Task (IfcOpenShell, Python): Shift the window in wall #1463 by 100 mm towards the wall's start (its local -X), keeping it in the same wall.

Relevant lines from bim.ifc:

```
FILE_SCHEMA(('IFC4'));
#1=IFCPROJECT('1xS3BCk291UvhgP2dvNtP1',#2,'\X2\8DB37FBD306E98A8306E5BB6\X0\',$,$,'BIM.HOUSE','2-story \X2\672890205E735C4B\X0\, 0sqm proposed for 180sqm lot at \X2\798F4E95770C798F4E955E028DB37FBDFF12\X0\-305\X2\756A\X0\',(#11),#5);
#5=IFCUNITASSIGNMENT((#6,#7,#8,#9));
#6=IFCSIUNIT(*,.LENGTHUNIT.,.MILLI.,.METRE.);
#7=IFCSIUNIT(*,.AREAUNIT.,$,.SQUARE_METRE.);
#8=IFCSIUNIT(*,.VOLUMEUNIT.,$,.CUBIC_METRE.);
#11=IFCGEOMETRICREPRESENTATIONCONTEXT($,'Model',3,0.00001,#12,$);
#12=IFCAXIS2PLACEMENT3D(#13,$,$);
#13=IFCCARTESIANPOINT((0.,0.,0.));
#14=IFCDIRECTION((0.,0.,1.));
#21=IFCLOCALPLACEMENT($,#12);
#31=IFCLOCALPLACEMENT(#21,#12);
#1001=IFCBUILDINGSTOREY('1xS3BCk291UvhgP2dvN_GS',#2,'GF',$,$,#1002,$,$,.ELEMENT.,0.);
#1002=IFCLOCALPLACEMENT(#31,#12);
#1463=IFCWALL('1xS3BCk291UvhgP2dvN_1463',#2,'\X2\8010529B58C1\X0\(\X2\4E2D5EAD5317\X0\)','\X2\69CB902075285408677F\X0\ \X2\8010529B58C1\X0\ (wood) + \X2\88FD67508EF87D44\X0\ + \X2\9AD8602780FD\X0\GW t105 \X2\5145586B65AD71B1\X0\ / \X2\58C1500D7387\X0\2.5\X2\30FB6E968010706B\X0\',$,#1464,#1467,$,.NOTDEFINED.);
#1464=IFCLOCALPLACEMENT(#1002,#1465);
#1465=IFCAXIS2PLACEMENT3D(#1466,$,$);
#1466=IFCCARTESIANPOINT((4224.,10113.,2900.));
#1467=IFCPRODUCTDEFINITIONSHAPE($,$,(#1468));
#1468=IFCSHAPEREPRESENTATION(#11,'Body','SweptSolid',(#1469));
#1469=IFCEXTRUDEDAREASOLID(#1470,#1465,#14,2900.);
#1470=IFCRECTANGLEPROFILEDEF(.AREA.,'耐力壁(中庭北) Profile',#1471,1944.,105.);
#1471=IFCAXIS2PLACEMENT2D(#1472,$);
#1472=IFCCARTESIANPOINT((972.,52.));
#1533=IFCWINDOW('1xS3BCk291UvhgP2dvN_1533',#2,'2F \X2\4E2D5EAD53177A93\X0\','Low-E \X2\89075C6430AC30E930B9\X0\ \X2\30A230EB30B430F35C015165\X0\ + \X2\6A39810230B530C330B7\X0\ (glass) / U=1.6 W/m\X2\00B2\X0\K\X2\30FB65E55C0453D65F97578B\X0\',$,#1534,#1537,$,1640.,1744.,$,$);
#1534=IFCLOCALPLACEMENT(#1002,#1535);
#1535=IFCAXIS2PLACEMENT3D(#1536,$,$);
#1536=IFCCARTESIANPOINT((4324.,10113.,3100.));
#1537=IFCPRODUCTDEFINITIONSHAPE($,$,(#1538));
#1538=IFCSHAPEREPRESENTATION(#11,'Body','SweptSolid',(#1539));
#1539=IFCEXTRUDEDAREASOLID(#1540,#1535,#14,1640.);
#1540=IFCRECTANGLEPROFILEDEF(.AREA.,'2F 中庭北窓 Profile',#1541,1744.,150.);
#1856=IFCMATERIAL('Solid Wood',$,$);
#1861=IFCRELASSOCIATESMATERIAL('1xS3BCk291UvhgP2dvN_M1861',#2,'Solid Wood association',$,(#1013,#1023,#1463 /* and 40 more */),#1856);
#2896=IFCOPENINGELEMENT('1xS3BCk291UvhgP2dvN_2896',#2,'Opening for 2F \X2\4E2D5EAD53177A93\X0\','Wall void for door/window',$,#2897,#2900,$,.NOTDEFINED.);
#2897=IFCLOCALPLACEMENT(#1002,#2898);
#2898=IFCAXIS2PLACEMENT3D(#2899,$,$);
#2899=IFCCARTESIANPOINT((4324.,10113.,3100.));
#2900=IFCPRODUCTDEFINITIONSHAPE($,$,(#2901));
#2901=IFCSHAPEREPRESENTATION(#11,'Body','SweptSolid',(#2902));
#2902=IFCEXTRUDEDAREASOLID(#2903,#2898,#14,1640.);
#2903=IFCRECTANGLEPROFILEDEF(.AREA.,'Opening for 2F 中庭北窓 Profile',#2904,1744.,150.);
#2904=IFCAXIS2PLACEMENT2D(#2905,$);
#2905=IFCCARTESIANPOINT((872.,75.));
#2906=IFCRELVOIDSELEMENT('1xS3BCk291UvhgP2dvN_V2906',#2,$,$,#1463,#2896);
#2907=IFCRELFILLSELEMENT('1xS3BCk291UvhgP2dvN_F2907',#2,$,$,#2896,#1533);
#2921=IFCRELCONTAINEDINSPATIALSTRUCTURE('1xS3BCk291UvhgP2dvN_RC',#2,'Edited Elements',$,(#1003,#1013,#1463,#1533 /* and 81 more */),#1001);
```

```python
import ifcopenshell
import ifcopenshell.api.geometry
import ifcopenshell.util.placement
import ifcopenshell.util.unit

model = ifcopenshell.open("bim.ifc")
unit_scale = ifcopenshell.util.unit.calculate_unit_scale(model)

window = model.by_id(1533)
opening = window.FillsVoids[0].RelatingOpeningElement
wall = opening.VoidsElements[0].RelatingBuildingElement

wall_matrix = ifcopenshell.util.placement.get_local_placement(wall.ObjectPlacement)
shift = wall_matrix[:3, 0] * -0.1 / unit_scale
before = ifcopenshell.util.placement.get_local_placement(window.ObjectPlacement)[:3, 3].copy()

# The window is not placed relative to its opening, so move both.
for product in (opening, window):
    matrix = ifcopenshell.util.placement.get_local_placement(product.ObjectPlacement)
    matrix[:3, 3] += shift
    ifcopenshell.api.geometry.edit_object_placement(model, product=product, matrix=matrix, is_si=False)

after = ifcopenshell.util.placement.get_local_placement(window.ObjectPlacement)[:3, 3]
print("window moved by", (after - before).round(3) + 0.0)

model.write("bim_updated.ifc")
```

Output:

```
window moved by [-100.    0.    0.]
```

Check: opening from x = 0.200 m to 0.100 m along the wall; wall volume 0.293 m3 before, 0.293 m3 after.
